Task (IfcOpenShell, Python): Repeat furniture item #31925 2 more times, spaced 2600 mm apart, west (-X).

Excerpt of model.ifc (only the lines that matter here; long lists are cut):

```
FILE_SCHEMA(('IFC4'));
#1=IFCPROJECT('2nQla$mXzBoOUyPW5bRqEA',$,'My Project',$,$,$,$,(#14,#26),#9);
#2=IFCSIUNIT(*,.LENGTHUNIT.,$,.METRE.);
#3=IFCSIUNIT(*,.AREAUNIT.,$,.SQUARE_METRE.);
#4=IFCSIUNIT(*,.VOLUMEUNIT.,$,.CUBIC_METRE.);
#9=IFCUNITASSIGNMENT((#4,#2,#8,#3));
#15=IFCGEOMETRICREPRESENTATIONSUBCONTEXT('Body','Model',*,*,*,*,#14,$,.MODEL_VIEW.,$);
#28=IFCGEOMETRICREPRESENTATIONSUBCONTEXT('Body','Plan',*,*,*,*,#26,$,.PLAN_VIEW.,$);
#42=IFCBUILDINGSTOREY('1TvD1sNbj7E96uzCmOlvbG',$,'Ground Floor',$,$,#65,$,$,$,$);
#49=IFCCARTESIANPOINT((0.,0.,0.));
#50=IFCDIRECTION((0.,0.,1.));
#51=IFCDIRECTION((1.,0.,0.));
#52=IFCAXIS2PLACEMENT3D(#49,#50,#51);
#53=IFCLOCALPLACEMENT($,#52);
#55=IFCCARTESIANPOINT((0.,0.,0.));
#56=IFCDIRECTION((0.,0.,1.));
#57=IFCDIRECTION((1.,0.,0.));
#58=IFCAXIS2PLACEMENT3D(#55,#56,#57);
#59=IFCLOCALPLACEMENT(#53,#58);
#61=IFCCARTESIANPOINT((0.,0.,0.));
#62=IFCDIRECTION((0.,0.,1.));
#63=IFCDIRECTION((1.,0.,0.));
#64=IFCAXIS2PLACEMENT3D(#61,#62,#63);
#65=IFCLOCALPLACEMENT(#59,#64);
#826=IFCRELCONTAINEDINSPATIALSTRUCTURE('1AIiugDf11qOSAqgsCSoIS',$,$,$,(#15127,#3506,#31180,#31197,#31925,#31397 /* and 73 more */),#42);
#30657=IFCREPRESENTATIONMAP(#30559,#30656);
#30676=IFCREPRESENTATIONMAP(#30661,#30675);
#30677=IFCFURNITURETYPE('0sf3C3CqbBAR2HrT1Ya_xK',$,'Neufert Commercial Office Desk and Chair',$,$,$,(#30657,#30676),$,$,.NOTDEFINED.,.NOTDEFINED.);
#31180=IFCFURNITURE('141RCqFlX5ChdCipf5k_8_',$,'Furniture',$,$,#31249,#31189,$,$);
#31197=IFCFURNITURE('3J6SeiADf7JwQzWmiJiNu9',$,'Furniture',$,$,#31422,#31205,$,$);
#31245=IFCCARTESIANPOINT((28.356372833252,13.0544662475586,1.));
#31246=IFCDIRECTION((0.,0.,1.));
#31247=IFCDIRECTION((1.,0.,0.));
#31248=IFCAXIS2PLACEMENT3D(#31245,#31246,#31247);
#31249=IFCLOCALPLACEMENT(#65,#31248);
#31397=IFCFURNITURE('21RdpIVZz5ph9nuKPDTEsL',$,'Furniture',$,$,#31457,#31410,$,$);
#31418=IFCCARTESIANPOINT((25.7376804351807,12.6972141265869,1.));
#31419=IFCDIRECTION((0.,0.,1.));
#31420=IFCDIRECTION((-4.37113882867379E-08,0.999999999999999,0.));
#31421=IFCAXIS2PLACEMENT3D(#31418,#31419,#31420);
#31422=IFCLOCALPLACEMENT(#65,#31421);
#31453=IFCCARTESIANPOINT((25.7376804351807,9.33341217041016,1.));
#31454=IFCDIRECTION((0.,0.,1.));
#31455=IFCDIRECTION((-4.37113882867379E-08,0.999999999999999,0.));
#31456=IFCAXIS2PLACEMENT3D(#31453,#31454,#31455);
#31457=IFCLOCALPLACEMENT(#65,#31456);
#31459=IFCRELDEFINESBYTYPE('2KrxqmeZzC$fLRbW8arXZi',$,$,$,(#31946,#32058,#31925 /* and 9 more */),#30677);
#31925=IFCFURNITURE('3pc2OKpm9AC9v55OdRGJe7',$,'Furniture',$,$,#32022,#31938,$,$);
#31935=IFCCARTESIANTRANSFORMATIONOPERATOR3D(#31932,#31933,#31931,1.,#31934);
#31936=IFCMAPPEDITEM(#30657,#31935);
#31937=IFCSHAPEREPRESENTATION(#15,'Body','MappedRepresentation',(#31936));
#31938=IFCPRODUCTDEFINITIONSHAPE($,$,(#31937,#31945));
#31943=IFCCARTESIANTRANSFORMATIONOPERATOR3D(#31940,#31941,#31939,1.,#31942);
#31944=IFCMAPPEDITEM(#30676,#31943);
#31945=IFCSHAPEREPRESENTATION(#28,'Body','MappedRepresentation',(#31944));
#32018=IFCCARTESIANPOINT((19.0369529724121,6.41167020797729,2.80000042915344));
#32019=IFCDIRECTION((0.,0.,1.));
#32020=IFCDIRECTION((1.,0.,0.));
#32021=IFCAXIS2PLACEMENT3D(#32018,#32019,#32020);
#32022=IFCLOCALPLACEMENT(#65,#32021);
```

```python
import numpy as np
import ifcopenshell
import ifcopenshell.api.geometry
import ifcopenshell.api.root
import ifcopenshell.util.element
import ifcopenshell.util.placement
import ifcopenshell.util.unit

model = ifcopenshell.open("model.ifc")
unit_scale = ifcopenshell.util.unit.calculate_unit_scale(model)

source = model.by_guid("3pc2OKpm9AC9v55OdRGJe7")
base = ifcopenshell.util.placement.get_local_placement(source.ObjectPlacement)
step = np.array([-1.0, 0.0, 0.0]) * 2.6 / unit_scale

for i in range(1, 3):
    copy = ifcopenshell.api.root.copy_class(model, product=source)
    copy.Representation = ifcopenshell.util.element.copy_deep(
        model, source.Representation, exclude=["IfcGeometricRepresentationContext", "IfcRepresentationMap"]
    )
    matrix = base.copy()
    matrix[:3, 3] += i * step
    print("added at", matrix[:3, 3].round(3) + 0.0)
    ifcopenshell.api.geometry.edit_object_placement(model, product=copy, matrix=matrix, is_si=False)

model.write("model_rev.ifc")
```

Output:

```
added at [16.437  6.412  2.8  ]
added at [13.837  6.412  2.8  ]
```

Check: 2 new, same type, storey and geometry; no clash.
